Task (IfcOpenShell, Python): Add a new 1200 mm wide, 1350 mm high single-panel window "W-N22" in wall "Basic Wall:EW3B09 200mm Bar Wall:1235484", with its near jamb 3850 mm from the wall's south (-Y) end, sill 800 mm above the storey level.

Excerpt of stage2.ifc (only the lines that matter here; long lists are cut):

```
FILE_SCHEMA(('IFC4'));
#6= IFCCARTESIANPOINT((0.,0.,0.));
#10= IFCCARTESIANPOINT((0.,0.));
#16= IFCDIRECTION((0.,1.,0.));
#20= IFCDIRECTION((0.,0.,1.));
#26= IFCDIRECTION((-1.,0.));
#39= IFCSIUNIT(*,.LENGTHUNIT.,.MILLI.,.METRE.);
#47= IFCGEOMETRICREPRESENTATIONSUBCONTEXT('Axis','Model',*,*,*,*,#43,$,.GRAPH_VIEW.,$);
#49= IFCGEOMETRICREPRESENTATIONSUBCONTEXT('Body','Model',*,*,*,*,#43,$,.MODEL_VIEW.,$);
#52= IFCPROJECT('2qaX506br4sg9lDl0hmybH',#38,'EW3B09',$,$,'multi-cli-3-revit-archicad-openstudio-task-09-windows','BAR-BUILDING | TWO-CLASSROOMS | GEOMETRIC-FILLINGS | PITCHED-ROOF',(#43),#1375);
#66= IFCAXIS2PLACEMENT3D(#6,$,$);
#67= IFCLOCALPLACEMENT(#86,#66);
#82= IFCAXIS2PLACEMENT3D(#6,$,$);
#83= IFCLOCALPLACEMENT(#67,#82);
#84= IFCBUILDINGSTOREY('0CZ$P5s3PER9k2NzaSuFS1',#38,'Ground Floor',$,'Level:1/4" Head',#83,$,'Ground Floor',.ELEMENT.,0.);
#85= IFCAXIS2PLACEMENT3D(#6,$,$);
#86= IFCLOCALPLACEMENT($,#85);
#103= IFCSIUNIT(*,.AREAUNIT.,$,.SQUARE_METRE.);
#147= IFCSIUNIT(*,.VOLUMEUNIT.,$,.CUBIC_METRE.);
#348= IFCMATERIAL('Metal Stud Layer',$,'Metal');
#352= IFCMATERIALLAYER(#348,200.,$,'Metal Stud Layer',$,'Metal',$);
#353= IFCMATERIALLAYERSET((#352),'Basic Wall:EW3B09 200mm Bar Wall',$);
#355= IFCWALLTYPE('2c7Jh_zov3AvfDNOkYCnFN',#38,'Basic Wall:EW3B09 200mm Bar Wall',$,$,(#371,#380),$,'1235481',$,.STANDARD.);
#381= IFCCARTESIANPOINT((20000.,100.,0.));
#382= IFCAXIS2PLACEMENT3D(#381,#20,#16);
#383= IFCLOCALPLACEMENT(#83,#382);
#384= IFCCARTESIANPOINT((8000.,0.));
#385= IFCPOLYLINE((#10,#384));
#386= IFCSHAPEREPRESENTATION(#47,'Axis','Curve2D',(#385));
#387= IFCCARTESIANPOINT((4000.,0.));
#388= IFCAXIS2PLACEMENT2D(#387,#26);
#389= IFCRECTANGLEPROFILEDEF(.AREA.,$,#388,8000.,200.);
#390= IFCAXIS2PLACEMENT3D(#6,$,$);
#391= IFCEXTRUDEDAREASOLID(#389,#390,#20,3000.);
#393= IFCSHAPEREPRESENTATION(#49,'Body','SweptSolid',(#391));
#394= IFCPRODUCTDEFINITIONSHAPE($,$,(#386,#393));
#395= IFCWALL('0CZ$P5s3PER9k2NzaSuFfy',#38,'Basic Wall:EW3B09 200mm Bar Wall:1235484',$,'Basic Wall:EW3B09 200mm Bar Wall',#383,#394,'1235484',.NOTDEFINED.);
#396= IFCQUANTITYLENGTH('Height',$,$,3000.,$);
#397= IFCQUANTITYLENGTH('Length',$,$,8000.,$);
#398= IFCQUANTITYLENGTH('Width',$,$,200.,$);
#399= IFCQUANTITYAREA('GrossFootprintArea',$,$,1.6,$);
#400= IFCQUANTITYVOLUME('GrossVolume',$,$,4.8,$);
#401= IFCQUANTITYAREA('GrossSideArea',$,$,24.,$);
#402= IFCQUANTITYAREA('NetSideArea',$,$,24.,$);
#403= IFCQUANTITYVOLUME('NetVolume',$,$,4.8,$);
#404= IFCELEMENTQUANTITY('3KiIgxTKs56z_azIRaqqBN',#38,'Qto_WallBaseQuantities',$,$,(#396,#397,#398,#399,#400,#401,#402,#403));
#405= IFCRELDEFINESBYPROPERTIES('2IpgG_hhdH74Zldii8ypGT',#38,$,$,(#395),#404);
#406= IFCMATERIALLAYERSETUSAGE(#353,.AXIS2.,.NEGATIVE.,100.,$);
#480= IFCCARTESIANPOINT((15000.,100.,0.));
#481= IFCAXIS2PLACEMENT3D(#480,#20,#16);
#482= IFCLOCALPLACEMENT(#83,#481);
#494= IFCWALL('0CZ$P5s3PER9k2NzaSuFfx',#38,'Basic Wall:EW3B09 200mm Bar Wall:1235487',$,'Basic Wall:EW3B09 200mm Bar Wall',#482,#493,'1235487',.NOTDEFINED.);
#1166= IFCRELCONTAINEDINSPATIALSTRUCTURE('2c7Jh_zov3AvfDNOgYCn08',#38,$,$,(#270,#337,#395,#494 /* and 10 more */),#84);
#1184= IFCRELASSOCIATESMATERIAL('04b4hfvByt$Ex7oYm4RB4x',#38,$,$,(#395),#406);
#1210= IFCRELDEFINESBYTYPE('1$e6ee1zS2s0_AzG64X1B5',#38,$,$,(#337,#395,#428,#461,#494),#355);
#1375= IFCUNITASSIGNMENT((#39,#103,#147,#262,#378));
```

```python
import numpy as np
import ifcopenshell
import ifcopenshell.api.feature
import ifcopenshell.api.geometry
import ifcopenshell.api.pset
import ifcopenshell.api.root
import ifcopenshell.api.spatial
import ifcopenshell.geom
import ifcopenshell.util.element
import ifcopenshell.util.placement
import ifcopenshell.util.representation
import ifcopenshell.util.shape
import ifcopenshell.util.unit

model = ifcopenshell.open("stage2.ifc")
unit_scale = ifcopenshell.util.unit.calculate_unit_scale(model)
area_scale = ifcopenshell.util.unit.calculate_unit_scale(model, "AREAUNIT")
volume_scale = ifcopenshell.util.unit.calculate_unit_scale(model, "VOLUMEUNIT")
settings = ifcopenshell.geom.settings()


def volume(element):
    """Net volume in cubic metres, openings subtracted."""
    shape = ifcopenshell.geom.create_shape(settings, element)
    return ifcopenshell.util.shape.get_volume(shape.geometry)


wall = model.by_guid("0CZ$P5s3PER9k2NzaSuFfy")
storey = ifcopenshell.util.element.get_container(wall, ifc_class="IfcBuildingStorey")
context = ifcopenshell.util.representation.get_context(model, "Model", "Body", "MODEL_VIEW")
before = volume(wall)

width, height, from_end, sill = 1.2, 1.35, 3.85, 0.8  # metres

# The wall runs along its own X axis, and the end named is its -X end.
wall_shape = ifcopenshell.geom.create_shape(settings, wall)
x, y, z = ifcopenshell.util.shape.get_vertices(wall_shape.geometry).T
start = x.min() + from_end
face, thickness = float(y.min()), float(y.max() - y.min())
wall_matrix = ifcopenshell.util.placement.get_local_placement(wall.ObjectPlacement)
level = ifcopenshell.util.placement.get_local_placement(storey.ObjectPlacement)[2, 3]


def in_wall(x, y):
    """Placement at x, y metres in the wall's axes, at sill height."""
    matrix = wall_matrix.copy()
    matrix[:, 3] = wall_matrix @ np.array([x / unit_scale, y / unit_scale, 0.0, 1.0])
    matrix[2, 3] = level + sill / unit_scale
    return matrix


# Opening: a box that overshoots both wall faces by 50 mm.
opening = ifcopenshell.api.root.create_entity(model, ifc_class="IfcOpeningElement", predefined_type="OPENING")
box = ifcopenshell.api.geometry.add_wall_representation(
    model, context=context, length=width, height=height, thickness=thickness + 0.1
)
ifcopenshell.api.geometry.assign_representation(model, product=opening, representation=box)
ifcopenshell.api.geometry.edit_object_placement(model, product=opening, matrix=in_wall(start, face - 0.05), is_si=False)
ifcopenshell.api.feature.add_feature(model, feature=opening, element=wall)

window = ifcopenshell.api.root.create_entity(model, ifc_class="IfcWindow", name="W-N22", predefined_type="WINDOW")
window.OverallWidth, window.OverallHeight = width / unit_scale, height / unit_scale
window.PartitioningType = "SINGLE_PANEL"
body = ifcopenshell.api.geometry.add_window_representation(
    model,
    context=context,
    overall_width=window.OverallWidth,
    overall_height=window.OverallHeight,
    partition_type="SINGLE_PANEL",
)
ifcopenshell.api.geometry.assign_representation(model, product=window, representation=body)
ifcopenshell.api.spatial.assign_container(model, products=[window], relating_structure=storey)
ifcopenshell.api.feature.add_filling(model, opening=opening, element=window)

# Centre the window in the wall's thickness.
ifcopenshell.api.geometry.edit_object_placement(model, product=window, matrix=in_wall(start, face), is_si=False)
window_shape = ifcopenshell.geom.create_shape(settings, window)
depth = ifcopenshell.util.shape.get_vertices(window_shape.geometry)[:, 1]
offset = face + thickness / 2 - (depth.min() + depth.max()) / 2
ifcopenshell.api.geometry.edit_object_placement(model, product=window, matrix=in_wall(start, offset), is_si=False)

after = volume(wall)

# Update the wall's stored quantities.
qto = model.by_id(ifcopenshell.util.element.get_pset(wall, "Qto_WallBaseQuantities", should_inherit=False)["id"])
ifcopenshell.api.pset.edit_qto(model, qto=qto, properties={
    "NetSideArea": after / thickness / area_scale,
    "NetVolume": after / volume_scale,
})

print(f"wall volume {before:.3f} -> {after:.3f} m3")

model.write("stage2_edited.ifc")
```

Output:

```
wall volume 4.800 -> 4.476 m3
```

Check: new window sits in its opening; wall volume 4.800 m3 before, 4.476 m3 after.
